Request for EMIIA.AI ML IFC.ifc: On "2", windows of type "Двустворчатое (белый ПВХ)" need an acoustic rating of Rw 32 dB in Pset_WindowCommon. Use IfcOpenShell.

First a look at what the model holds.

```python
import ifcopenshell
import ifcopenshell.util.element

model = ifcopenshell.open("EMIIA.AI ML IFC.ifc")
print(model.schema)
storey = next(s for s in model.by_type("IfcBuildingStorey") if s.Name == "2")
windows = [e for e in ifcopenshell.util.element.get_decomposition(storey) if e.is_a("IfcWindow")]
seen = {}
for e in windows:
    element_type = ifcopenshell.util.element.get_type(e)
    key = (element_type.Name if element_type != e and element_type else None, ifcopenshell.util.element.get_pset(e, "Pset_WindowCommon", "AcousticRating"))
    seen[key] = seen.get(key, 0) + 1
for (name, value), count in sorted(seen.items(), key=str):
    print(count, "x", name, "|", value)
```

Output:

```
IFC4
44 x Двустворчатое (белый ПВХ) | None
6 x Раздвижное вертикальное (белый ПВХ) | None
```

```python
import ifcopenshell
import ifcopenshell.api.pset
import ifcopenshell.util.element

model = ifcopenshell.open("EMIIA.AI ML IFC.ifc")

storey = next(s for s in model.by_type("IfcBuildingStorey") if s.Name == "2")
windows = [e for e in ifcopenshell.util.element.get_decomposition(storey) if e.is_a("IfcWindow")]

count = 0
for e in windows:
    element_type = ifcopenshell.util.element.get_type(e)
    if element_type in (None, e) or element_type.Name != "Двустворчатое (белый ПВХ)":
        continue
    # add_pset returns the element's existing set when there is one.
    pset = ifcopenshell.api.pset.add_pset(model, product=e, name="Pset_WindowCommon")
    ifcopenshell.api.pset.edit_pset(model, pset=pset, properties={"AcousticRating": "Rw 32 dB"})
    count += 1

print(count, "windows updated")

model.write("EMIIA.AI ML IFC_rev.ifc")
```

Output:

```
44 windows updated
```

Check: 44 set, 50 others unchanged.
